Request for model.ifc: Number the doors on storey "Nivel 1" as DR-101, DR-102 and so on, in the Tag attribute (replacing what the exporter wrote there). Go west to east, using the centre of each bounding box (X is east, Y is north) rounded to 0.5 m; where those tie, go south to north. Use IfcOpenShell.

First a look at what the model holds.

```python
import ifcopenshell
import ifcopenshell.util.element
import ifcopenshell.util.placement

model = ifcopenshell.open("model.ifc")
print(model.schema)
storey = next(s for s in model.by_type("IfcBuildingStorey") if s.Name == "Nivel 1")
doors = [e for e in ifcopenshell.util.element.get_decomposition(storey) if e.is_a("IfcDoor")]
for e in sorted(doors, key=lambda e: e.id()):
    origin = ifcopenshell.util.placement.get_local_placement(e.ObjectPlacement)[:3, 3]
    print(e.id(), e.Tag, e.Name, origin.round(2) + 0.0, sep=" | ")
```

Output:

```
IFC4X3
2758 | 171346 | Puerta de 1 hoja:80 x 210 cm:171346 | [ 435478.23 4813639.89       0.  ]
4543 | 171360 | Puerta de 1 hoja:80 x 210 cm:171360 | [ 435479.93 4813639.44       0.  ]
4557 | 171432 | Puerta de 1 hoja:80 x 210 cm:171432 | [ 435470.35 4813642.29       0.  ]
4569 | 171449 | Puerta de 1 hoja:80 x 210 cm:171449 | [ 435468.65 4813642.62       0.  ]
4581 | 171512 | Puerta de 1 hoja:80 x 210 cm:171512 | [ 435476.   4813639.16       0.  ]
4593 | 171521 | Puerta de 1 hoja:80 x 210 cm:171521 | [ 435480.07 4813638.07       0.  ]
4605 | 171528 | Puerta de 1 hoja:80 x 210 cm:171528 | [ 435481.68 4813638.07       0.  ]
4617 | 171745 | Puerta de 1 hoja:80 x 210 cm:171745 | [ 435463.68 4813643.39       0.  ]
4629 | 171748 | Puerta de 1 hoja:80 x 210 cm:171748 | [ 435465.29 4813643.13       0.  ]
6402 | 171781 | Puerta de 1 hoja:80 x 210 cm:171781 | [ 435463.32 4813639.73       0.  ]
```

```python
import ifcopenshell
import ifcopenshell.geom
import ifcopenshell.util.element
import ifcopenshell.util.shape

model = ifcopenshell.open("model.ifc")
settings = ifcopenshell.geom.settings()
settings.set("use-world-coords", True)


def centre(element):
    shape = ifcopenshell.geom.create_shape(settings, element)
    return ifcopenshell.util.shape.get_bbox_centroid(shape.geometry)


storey = next(s for s in model.by_type("IfcBuildingStorey") if s.Name == "Nivel 1")
doors = [e for e in ifcopenshell.util.element.get_decomposition(storey) if e.is_a("IfcDoor")]

# Insertion points can sit at a corner or the storey origin, so sort by the geometry (in metres).
centres = {e: centre(e) for e in doors}
doors.sort(key=lambda e: (round(centres[e][0] / 0.5), centres[e][1]))

for i, e in enumerate(doors, start=1):
    number = f"DR-1{i:02d}"
    e.Tag = number
    print(e.id(), number)

model.write("model_updated.ifc")
```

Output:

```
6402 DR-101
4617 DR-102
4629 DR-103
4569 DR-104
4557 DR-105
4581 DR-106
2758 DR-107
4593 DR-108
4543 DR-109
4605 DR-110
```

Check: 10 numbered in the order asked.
